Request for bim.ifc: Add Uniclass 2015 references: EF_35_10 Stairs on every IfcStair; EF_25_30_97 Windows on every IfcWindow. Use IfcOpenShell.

First a look at what the model holds.

```python
import ifcopenshell

model = ifcopenshell.open("bim.ifc")
print(model.schema)
print("classifications:", [c.Name for c in model.by_type("IfcClassification")])
for ifc_class in ("IfcDoor", "IfcRoof", "IfcStair", "IfcWall", "IfcWindow"):
    print(ifc_class, len(model.by_type(ifc_class)))
```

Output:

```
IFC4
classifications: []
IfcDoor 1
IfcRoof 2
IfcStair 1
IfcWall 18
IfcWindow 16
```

```python
import ifcopenshell
import ifcopenshell.api.classification

model = ifcopenshell.open("bim.ifc")

system = ifcopenshell.api.classification.add_classification(model, classification="Uniclass 2015")

codes = {
    "IfcStair": ("EF_35_10", "Stairs"),
    "IfcWindow": ("EF_25_30_97", "Windows"),
}
for ifc_class, (code, name) in codes.items():
    products = model.by_type(ifc_class)
    ifcopenshell.api.classification.add_reference(
        model, products=products, classification=system, identification=code, name=name
    )
    print(code, len(products))

model.write("bim-out.ifc")
```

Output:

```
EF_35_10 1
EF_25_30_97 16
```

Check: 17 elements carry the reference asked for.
